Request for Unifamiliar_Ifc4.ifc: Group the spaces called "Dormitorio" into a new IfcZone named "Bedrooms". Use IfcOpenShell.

First a look at what the model holds.

```python
import ifcopenshell

model = ifcopenshell.open("Unifamiliar_Ifc4.ifc")
print(model.schema)
seen = {}
for space in model.by_type("IfcSpace"):
    seen[space.LongName] = seen.get(space.LongName, 0) + 1
for name, count in sorted(seen.items(), key=str):
    print(count, "x", name)
print("zones:", [z.Name for z in model.by_type("IfcZone")][:20])
```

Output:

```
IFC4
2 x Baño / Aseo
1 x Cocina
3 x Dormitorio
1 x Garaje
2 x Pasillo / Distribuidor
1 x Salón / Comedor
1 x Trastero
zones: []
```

```python
import ifcopenshell
import ifcopenshell.api.group
import ifcopenshell.api.root

model = ifcopenshell.open("Unifamiliar_Ifc4.ifc")

names = {"Dormitorio"}
spaces = [s for s in model.by_type("IfcSpace") if s.LongName in names]

zone = ifcopenshell.api.root.create_entity(model, ifc_class="IfcZone", name="Bedrooms")
ifcopenshell.api.group.assign_group(model, products=spaces, group=zone)
print(len(spaces), "spaces in", zone.Name)

model.write("Unifamiliar_Ifc4_v2.ifc")
```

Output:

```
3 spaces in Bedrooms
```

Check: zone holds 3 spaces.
